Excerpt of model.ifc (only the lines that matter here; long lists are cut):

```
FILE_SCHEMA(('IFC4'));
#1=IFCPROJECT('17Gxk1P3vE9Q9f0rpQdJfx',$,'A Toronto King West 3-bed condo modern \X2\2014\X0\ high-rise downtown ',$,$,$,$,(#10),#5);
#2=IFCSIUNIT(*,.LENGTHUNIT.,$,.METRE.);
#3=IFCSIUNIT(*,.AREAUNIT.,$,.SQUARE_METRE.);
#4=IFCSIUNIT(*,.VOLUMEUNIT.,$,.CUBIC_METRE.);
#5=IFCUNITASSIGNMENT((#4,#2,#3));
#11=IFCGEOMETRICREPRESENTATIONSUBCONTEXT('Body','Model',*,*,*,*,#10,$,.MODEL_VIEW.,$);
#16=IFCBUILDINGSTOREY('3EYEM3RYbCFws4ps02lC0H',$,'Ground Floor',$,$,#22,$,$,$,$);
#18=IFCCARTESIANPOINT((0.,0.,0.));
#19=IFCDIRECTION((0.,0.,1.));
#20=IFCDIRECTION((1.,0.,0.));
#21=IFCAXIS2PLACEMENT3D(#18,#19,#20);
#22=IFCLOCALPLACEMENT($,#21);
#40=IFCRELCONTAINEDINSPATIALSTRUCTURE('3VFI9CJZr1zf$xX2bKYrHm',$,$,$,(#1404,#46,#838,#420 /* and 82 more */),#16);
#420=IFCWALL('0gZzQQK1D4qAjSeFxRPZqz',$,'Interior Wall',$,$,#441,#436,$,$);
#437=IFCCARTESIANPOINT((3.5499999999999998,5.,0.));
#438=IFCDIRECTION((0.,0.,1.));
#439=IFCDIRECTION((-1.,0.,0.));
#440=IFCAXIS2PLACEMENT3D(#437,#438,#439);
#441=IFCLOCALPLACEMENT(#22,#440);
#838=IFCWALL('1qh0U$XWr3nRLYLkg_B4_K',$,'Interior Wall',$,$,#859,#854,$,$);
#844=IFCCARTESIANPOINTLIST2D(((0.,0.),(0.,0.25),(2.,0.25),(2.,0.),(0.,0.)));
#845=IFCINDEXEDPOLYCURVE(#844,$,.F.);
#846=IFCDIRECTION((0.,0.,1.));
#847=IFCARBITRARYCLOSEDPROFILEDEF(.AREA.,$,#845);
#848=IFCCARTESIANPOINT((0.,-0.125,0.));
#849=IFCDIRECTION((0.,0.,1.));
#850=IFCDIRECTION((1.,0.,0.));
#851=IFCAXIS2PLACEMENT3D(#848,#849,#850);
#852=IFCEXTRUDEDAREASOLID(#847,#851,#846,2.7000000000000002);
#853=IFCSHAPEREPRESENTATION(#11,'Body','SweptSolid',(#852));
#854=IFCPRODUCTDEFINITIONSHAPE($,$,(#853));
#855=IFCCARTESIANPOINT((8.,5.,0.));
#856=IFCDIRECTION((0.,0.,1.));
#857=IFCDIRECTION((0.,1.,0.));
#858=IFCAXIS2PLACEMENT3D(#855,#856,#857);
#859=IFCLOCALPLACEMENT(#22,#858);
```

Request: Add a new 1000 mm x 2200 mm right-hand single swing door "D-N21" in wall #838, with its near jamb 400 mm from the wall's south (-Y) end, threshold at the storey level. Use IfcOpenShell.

```python
import numpy as np
import ifcopenshell
import ifcopenshell.api.feature
import ifcopenshell.api.geometry
import ifcopenshell.api.root
import ifcopenshell.api.spatial
import ifcopenshell.geom
import ifcopenshell.util.element
import ifcopenshell.util.placement
import ifcopenshell.util.representation
import ifcopenshell.util.shape
import ifcopenshell.util.unit

model = ifcopenshell.open("model.ifc")
unit_scale = ifcopenshell.util.unit.calculate_unit_scale(model)
settings = ifcopenshell.geom.settings()


def volume(element):
    """Net volume in cubic metres, openings subtracted."""
    shape = ifcopenshell.geom.create_shape(settings, element)
    return ifcopenshell.util.shape.get_volume(shape.geometry)


wall = model.by_guid("1qh0U$XWr3nRLYLkg_B4_K")
storey = ifcopenshell.util.element.get_container(wall, ifc_class="IfcBuildingStorey")
context = ifcopenshell.util.representation.get_context(model, "Model", "Body", "MODEL_VIEW")
before = volume(wall)

width, height, from_end, sill = 1, 2.2, 0.4, 0.0  # metres

# The wall runs along its own X axis, and the end named is its -X end.
wall_shape = ifcopenshell.geom.create_shape(settings, wall)
x, y, z = ifcopenshell.util.shape.get_vertices(wall_shape.geometry).T
start = x.min() + from_end
face, thickness = float(y.min()), float(y.max() - y.min())
wall_matrix = ifcopenshell.util.placement.get_local_placement(wall.ObjectPlacement)
level = ifcopenshell.util.placement.get_local_placement(storey.ObjectPlacement)[2, 3]


def in_wall(x, y):
    """Placement at x, y metres in the wall's axes, at sill height."""
    matrix = wall_matrix.copy()
    matrix[:, 3] = wall_matrix @ np.array([x / unit_scale, y / unit_scale, 0.0, 1.0])
    matrix[2, 3] = level + sill / unit_scale
    return matrix


# Opening: a box that overshoots both wall faces by 50 mm.
opening = ifcopenshell.api.root.create_entity(model, ifc_class="IfcOpeningElement", predefined_type="OPENING")
box = ifcopenshell.api.geometry.add_wall_representation(
    model, context=context, length=width, height=height, thickness=thickness + 0.1
)
ifcopenshell.api.geometry.assign_representation(model, product=opening, representation=box)
ifcopenshell.api.geometry.edit_object_placement(model, product=opening, matrix=in_wall(start, face - 0.05), is_si=False)
ifcopenshell.api.feature.add_feature(model, feature=opening, element=wall)

door = ifcopenshell.api.root.create_entity(model, ifc_class="IfcDoor", name="D-N21", predefined_type="DOOR")
door.OverallWidth, door.OverallHeight = width / unit_scale, height / unit_scale
door.OperationType = "SINGLE_SWING_RIGHT"
body = ifcopenshell.api.geometry.add_door_representation(
    model,
    context=context,
    overall_width=door.OverallWidth,
    overall_height=door.OverallHeight,
    operation_type="SINGLE_SWING_RIGHT",
    lining_properties={"LiningDepth": thickness / unit_scale, "ThresholdDepth": thickness / unit_scale},
)
ifcopenshell.api.geometry.assign_representation(model, product=door, representation=body)
ifcopenshell.api.spatial.assign_container(model, products=[door], relating_structure=storey)
ifcopenshell.api.feature.add_filling(model, opening=opening, element=door)

# The lining spans the wall, so the door starts at the wall face.
ifcopenshell.api.geometry.edit_object_placement(model, product=door, matrix=in_wall(start, face), is_si=False)

after = volume(wall)

print(f"wall volume {before:.3f} -> {after:.3f} m3")

model.write("model_edited.ifc")
```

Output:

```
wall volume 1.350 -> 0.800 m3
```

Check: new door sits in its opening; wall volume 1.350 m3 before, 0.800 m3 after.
